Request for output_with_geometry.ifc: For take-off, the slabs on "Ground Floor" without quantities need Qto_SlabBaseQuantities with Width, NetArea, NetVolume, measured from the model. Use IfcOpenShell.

First a look at what the model holds.

```python
import ifcopenshell
import ifcopenshell.util.element
import ifcopenshell.util.unit

model = ifcopenshell.open("output_with_geometry.ifc")
print(model.schema)
for unit_type in ("LENGTHUNIT", "AREAUNIT", "VOLUMEUNIT"):
    print(unit_type, ifcopenshell.util.unit.calculate_unit_scale(model, unit_type))
storey = next(s for s in model.by_type("IfcBuildingStorey") if s.Name == "Ground Floor")
slabs = [e for e in ifcopenshell.util.element.get_decomposition(storey) if e.is_a("IfcSlab")]
for e in sorted(slabs, key=lambda e: e.id()):
    print(e.id(), e.is_a(), e.Name, list(ifcopenshell.util.element.get_psets(e, qtos_only=True)), sep=" | ")
```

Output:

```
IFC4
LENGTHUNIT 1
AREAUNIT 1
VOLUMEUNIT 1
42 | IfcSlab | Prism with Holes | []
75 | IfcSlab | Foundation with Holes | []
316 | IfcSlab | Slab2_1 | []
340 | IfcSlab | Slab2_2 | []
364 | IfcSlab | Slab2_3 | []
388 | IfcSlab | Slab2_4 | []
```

```python
import ifcopenshell
import ifcopenshell.api.pset
import ifcopenshell.geom
import ifcopenshell.util.element
import ifcopenshell.util.shape
import ifcopenshell.util.unit

model = ifcopenshell.open("output_with_geometry.ifc")
unit_scale = ifcopenshell.util.unit.calculate_unit_scale(model)
area_scale = ifcopenshell.util.unit.calculate_unit_scale(model, "AREAUNIT")
volume_scale = ifcopenshell.util.unit.calculate_unit_scale(model, "VOLUMEUNIT")
settings = ifcopenshell.geom.settings()

storey = next(s for s in model.by_type("IfcBuildingStorey") if s.Name == "Ground Floor")
slabs = [e for e in ifcopenshell.util.element.get_decomposition(storey) if e.is_a("IfcSlab")]

for e in sorted(slabs, key=lambda e: e.id()):
    if ifcopenshell.util.element.get_psets(e, qtos_only=True, should_inherit=False):
        continue
    # Geometry comes back in metres, in the element's own axes.
    shape = ifcopenshell.geom.create_shape(settings, e)
    values = {
        "Width": ifcopenshell.util.shape.get_z(shape.geometry) / unit_scale,
        "NetArea": ifcopenshell.util.shape.get_footprint_area(shape.geometry) / area_scale,
        "NetVolume": ifcopenshell.util.shape.get_volume(shape.geometry) / volume_scale,
    }
    qto = ifcopenshell.api.pset.add_qto(model, product=e, name="Qto_SlabBaseQuantities")
    ifcopenshell.api.pset.edit_qto(model, qto=qto, properties=values)
    print(e.id(), {k: round(v, 3) for k, v in values.items()})

model.write("output_with_geometry-out.ifc")
```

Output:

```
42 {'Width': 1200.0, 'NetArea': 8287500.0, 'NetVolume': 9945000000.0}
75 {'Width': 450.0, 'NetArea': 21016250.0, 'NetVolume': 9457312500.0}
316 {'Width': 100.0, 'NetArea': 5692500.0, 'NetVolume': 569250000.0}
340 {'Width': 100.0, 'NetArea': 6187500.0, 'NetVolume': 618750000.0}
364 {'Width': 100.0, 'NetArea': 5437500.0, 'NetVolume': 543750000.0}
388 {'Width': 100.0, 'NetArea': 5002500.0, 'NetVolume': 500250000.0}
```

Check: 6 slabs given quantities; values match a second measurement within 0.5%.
